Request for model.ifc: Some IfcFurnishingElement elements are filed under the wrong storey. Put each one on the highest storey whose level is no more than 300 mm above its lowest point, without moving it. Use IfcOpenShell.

First a look at what the model holds.

```python
import ifcopenshell
import ifcopenshell.util.element
import ifcopenshell.util.placement

model = ifcopenshell.open("model.ifc")
print(model.schema)
for storey in model.by_type("IfcBuildingStorey"):
    level = ifcopenshell.util.placement.get_storey_elevation(storey)
    count = sum(e.is_a("IfcFurnishingElement") for e in ifcopenshell.util.element.get_contained(storey))
    print(storey.id(), storey.Name, round(level, 3), count, sep=" | ")
```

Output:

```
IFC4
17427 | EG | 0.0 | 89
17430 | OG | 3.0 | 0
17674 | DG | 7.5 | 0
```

```python
import ifcopenshell
import ifcopenshell.api.spatial
import ifcopenshell.geom
import ifcopenshell.util.element
import ifcopenshell.util.placement
import ifcopenshell.util.shape
import ifcopenshell.util.unit

model = ifcopenshell.open("model.ifc")
unit_scale = ifcopenshell.util.unit.calculate_unit_scale(model)
settings = ifcopenshell.geom.settings()

levels = sorted(
    ((ifcopenshell.util.placement.get_storey_elevation(s) * unit_scale, s) for s in model.by_type("IfcBuildingStorey")),
    key=lambda pair: pair[0],
)

for e in model.by_type("IfcFurnishingElement"):
    current = e.ContainedInStructure[0].RelatingStructure if e.ContainedInStructure else None
    if current is None or not current.is_a("IfcBuildingStorey"):
        continue
    shape = ifcopenshell.geom.create_shape(settings, e)
    bottom = ifcopenshell.util.shape.get_shape_bottom_elevation(shape, shape.geometry)
    below = [s for level, s in levels if level <= bottom + 0.3]
    storey = below[-1] if below else levels[0][1]
    if storey != current:
        # assign_container keeps the world position.
        ifcopenshell.api.spatial.assign_container(model, products=[e], relating_structure=storey)
        print(e.id(), current.Name, "->", storey.Name)

model.write("model_rev.ifc")
```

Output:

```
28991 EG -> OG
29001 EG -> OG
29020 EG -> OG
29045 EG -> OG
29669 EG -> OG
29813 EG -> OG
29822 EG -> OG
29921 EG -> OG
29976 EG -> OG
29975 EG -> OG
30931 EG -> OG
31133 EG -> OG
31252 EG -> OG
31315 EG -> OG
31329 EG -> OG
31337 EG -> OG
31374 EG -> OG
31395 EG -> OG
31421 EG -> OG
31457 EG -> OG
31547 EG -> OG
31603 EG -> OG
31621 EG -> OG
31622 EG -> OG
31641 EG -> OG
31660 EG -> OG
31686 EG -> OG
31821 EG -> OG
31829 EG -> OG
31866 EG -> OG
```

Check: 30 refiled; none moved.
